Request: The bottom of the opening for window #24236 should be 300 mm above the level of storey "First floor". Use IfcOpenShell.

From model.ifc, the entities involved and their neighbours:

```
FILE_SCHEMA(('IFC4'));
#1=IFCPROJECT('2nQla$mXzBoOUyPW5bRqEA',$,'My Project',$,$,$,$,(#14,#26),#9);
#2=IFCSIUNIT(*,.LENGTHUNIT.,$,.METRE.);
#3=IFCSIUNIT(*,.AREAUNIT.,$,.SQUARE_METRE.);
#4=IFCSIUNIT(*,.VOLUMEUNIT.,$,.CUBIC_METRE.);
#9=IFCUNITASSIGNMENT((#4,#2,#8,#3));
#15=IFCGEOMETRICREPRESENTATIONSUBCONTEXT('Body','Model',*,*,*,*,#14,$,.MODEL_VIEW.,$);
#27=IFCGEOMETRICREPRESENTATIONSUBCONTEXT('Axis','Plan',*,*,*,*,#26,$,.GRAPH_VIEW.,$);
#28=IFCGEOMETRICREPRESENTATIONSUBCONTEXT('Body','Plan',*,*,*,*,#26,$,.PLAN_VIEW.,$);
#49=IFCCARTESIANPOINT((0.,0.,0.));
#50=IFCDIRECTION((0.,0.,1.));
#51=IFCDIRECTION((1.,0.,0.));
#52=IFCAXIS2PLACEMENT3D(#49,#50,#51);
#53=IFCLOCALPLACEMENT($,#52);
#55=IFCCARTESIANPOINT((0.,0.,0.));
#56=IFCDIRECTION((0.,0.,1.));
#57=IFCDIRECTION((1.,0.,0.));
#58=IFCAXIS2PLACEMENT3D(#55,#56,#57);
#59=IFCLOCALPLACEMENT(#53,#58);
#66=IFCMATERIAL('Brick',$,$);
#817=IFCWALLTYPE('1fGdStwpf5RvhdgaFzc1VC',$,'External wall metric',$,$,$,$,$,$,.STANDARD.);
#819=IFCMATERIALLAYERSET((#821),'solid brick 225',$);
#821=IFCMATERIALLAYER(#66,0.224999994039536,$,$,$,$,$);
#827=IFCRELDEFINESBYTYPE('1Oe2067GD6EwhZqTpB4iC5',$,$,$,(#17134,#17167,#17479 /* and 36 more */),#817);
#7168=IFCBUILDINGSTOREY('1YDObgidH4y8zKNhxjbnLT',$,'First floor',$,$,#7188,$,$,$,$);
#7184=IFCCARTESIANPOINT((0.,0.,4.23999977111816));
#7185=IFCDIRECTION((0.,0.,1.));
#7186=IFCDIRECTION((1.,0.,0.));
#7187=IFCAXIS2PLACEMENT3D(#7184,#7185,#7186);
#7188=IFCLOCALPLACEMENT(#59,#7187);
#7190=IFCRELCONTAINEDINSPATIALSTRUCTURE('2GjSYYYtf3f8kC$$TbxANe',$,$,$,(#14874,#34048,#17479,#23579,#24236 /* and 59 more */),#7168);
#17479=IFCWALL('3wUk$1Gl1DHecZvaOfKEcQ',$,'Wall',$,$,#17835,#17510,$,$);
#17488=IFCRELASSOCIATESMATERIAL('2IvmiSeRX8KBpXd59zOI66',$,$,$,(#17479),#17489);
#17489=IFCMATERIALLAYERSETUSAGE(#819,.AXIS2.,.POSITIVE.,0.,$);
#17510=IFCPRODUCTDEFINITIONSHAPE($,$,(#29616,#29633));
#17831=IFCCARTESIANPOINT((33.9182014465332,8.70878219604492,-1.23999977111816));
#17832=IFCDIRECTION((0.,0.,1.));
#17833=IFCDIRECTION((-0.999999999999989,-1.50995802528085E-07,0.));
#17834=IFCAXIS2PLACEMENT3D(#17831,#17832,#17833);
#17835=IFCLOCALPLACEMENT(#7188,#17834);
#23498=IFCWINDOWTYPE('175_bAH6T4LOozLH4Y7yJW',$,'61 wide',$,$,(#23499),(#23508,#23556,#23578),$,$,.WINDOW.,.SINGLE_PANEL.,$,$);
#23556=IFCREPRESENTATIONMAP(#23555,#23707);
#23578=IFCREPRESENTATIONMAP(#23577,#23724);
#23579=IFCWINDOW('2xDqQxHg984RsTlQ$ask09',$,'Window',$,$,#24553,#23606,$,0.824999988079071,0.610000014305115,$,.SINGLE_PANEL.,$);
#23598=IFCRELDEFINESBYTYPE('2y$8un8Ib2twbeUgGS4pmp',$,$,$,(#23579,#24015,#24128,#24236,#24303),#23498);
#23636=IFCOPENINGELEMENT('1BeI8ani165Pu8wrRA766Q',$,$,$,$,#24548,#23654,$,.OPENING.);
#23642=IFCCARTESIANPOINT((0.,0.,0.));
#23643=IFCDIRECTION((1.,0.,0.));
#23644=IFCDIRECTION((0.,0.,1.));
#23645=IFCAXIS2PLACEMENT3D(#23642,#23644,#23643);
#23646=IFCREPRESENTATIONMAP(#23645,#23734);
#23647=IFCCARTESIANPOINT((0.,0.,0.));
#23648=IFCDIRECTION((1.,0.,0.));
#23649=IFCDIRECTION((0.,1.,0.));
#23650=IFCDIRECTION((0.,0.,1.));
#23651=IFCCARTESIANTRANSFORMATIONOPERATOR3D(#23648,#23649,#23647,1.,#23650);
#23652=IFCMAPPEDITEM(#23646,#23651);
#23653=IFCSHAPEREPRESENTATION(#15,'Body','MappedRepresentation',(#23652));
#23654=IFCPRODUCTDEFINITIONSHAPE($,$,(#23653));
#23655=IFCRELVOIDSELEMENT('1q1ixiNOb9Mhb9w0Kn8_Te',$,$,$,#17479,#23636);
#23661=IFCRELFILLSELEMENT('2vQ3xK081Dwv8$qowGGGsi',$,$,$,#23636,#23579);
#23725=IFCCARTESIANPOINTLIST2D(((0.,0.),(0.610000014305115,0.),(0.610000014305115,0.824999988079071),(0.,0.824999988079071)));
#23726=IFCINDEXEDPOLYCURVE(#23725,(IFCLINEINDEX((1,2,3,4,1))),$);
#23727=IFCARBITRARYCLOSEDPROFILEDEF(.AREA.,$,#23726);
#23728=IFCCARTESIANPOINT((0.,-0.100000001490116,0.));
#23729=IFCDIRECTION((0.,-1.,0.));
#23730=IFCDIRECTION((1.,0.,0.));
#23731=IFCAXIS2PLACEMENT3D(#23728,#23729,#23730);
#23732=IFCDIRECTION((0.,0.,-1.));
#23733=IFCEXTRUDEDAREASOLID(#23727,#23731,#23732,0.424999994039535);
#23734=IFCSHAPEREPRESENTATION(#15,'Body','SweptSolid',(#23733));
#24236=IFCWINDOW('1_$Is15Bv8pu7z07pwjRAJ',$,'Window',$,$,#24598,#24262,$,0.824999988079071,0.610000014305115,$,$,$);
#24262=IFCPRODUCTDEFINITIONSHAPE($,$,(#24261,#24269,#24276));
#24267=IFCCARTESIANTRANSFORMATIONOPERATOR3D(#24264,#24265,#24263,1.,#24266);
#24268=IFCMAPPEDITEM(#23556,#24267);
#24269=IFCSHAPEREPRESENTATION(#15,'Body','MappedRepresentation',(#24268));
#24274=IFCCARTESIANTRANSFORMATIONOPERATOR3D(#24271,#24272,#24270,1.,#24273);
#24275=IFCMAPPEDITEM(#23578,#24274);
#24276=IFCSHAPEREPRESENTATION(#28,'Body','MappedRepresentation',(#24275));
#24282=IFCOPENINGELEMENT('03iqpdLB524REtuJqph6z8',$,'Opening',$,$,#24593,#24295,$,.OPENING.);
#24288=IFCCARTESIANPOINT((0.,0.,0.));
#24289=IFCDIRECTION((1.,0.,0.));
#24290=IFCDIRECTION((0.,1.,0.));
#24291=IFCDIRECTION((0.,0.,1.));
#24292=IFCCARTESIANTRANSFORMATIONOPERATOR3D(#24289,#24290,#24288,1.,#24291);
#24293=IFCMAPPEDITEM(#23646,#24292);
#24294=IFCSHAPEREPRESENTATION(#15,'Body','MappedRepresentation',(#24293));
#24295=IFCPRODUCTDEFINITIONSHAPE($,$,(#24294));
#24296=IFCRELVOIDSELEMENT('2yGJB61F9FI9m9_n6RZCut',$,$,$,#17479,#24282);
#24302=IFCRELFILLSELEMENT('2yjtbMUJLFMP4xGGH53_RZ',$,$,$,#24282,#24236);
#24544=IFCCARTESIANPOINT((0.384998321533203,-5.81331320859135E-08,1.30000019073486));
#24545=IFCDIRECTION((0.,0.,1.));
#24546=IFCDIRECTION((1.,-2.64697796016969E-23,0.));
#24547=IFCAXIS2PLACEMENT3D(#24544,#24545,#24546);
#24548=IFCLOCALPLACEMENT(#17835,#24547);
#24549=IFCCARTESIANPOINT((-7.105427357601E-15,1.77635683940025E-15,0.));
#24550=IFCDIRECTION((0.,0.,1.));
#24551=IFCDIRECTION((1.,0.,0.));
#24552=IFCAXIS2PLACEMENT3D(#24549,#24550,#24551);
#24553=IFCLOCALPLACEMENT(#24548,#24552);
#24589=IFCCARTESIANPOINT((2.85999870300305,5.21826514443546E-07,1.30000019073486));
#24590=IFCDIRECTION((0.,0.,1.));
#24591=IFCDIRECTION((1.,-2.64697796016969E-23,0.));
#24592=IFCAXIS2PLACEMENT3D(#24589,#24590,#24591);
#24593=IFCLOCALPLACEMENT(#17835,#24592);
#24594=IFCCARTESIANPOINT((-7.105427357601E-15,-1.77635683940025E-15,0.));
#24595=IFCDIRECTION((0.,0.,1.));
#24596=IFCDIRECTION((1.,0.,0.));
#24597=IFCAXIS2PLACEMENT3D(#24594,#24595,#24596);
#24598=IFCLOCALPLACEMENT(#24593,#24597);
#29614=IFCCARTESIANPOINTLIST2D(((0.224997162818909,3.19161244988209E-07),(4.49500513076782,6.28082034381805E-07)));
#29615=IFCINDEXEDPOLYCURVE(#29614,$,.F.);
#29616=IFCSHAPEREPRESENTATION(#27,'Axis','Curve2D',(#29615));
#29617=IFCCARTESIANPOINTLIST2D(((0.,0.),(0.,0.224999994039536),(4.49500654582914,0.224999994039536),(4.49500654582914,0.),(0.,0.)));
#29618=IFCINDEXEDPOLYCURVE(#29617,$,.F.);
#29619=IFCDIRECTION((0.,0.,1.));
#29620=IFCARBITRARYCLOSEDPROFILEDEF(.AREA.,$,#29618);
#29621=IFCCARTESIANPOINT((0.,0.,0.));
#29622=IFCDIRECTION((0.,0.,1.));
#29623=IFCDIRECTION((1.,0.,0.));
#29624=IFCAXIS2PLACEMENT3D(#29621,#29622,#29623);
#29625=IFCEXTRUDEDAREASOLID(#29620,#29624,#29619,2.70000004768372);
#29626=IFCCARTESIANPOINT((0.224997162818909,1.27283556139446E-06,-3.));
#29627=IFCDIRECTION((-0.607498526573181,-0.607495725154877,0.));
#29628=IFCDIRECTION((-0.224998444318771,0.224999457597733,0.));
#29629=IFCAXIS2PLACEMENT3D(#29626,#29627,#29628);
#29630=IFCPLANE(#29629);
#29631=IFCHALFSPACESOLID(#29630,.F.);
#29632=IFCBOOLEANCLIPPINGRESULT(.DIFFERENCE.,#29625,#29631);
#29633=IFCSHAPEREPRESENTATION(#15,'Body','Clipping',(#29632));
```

```python
import numpy as np
import ifcopenshell
import ifcopenshell.api.geometry
import ifcopenshell.geom
import ifcopenshell.util.element
import ifcopenshell.util.placement
import ifcopenshell.util.shape
import ifcopenshell.util.unit

model = ifcopenshell.open("model.ifc")
unit_scale = ifcopenshell.util.unit.calculate_unit_scale(model)

window = model.by_guid("1_$Is15Bv8pu7z07pwjRAJ")
opening = window.FillsVoids[0].RelatingOpeningElement
storey = ifcopenshell.util.element.get_container(window, ifc_class="IfcBuildingStorey")
level = ifcopenshell.util.placement.get_local_placement(storey.ObjectPlacement)[2, 3]

# The opening's origin need not be at the sill, so measure its lowest point.
shape = ifcopenshell.geom.create_shape(ifcopenshell.geom.settings(), opening)
bottom = ifcopenshell.util.shape.get_shape_bottom_elevation(shape, shape.geometry) / unit_scale
dz = level + 0.3 / unit_scale - bottom

shift = np.array([0.0, 0.0, dz])
# The window is placed relative to its opening, so it follows when the opening moves.
matrix = ifcopenshell.util.placement.get_local_placement(opening.ObjectPlacement)
matrix[:3, 3] += shift
ifcopenshell.api.geometry.edit_object_placement(
    model, product=opening, matrix=matrix, is_si=False, should_transform_children=True
)

print(f"moved by {dz * unit_scale:+.3f} m")

model.write("model_v2.ifc")
```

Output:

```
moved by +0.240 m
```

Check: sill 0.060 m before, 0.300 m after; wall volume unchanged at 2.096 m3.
